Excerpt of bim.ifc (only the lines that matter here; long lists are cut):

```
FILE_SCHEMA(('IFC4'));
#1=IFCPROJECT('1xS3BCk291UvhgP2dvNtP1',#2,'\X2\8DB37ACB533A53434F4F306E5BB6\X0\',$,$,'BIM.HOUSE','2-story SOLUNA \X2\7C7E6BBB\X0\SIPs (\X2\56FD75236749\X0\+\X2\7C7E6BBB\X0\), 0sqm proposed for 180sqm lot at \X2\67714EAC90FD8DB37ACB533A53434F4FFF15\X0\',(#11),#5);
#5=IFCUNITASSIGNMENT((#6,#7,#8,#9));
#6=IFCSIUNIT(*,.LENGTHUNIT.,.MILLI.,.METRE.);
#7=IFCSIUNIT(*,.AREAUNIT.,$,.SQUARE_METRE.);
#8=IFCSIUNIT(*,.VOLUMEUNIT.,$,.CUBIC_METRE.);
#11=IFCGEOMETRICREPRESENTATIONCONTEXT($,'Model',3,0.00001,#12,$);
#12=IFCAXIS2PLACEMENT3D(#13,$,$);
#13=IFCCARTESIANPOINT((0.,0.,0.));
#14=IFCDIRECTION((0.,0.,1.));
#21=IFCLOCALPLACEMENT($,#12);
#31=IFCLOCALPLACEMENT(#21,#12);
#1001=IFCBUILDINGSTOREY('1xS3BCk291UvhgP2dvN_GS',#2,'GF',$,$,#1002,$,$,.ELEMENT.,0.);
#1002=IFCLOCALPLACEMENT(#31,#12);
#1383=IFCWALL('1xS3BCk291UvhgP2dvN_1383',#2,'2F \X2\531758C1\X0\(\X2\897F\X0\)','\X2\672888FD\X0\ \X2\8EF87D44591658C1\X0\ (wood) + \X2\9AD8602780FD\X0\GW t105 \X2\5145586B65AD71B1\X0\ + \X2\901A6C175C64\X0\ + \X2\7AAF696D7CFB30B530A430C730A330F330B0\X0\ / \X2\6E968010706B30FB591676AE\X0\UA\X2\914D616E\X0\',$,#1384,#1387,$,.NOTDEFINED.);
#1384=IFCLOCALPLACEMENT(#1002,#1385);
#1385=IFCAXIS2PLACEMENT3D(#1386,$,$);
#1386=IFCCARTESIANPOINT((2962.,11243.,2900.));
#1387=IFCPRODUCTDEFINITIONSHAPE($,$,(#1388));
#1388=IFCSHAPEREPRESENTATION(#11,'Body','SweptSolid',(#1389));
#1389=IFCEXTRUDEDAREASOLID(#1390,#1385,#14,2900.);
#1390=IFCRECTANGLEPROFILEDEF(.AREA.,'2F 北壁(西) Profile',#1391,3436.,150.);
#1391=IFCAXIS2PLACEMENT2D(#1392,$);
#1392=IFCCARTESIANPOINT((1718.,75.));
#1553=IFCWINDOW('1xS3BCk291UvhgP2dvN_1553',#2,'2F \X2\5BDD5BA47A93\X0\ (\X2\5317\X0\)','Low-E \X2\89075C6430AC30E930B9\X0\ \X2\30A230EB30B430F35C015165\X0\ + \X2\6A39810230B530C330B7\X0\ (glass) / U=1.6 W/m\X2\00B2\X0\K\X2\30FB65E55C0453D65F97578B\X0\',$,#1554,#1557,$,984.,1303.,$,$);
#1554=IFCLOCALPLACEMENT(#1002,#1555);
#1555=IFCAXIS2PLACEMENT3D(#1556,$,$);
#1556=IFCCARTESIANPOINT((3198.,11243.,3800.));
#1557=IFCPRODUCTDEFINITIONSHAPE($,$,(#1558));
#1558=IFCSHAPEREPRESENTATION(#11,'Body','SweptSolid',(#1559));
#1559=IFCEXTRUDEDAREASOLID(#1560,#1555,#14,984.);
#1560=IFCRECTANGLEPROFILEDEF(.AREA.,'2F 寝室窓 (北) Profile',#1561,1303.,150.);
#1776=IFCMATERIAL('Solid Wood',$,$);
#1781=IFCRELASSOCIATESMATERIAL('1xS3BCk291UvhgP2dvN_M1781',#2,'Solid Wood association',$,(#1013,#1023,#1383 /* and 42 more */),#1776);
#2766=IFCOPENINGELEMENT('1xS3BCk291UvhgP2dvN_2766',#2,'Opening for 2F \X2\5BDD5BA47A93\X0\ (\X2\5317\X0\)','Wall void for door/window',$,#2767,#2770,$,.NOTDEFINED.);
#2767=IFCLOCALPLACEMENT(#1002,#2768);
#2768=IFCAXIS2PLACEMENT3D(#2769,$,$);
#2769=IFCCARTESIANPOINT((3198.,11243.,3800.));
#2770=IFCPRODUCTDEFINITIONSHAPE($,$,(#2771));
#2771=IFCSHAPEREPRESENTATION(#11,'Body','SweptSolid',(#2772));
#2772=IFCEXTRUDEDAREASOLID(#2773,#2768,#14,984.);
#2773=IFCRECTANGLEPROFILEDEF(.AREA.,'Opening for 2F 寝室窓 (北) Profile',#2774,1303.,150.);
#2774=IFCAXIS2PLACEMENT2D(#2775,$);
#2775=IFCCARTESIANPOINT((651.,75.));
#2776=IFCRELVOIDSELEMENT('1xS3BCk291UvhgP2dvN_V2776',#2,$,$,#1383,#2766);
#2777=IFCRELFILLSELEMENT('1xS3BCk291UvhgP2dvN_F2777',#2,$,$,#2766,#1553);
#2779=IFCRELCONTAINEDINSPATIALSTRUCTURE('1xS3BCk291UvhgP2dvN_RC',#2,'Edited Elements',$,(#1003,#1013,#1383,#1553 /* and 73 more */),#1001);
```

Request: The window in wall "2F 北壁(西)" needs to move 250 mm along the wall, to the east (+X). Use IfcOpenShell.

```python
import ifcopenshell
import ifcopenshell.api.geometry
import ifcopenshell.util.placement

model = ifcopenshell.open("bim.ifc")

window = model.by_guid("1xS3BCk291UvhgP2dvN_1553")
opening = window.FillsVoids[0].RelatingOpeningElement
wall = opening.VoidsElements[0].RelatingBuildingElement

wall_matrix = ifcopenshell.util.placement.get_local_placement(wall.ObjectPlacement)
shift = wall_matrix[:3, 0] * 250.0
before = ifcopenshell.util.placement.get_local_placement(window.ObjectPlacement)[:3, 3].copy()

# The window is not placed relative to its opening, so move both.
for product in (opening, window):
    matrix = ifcopenshell.util.placement.get_local_placement(product.ObjectPlacement)
    matrix[:3, 3] += shift
    ifcopenshell.api.geometry.edit_object_placement(model, product=product, matrix=matrix, is_si=False)

after = ifcopenshell.util.placement.get_local_placement(window.ObjectPlacement)[:3, 3]
print("window moved by", (after - before).round(3) + 0.0)

model.write("bim_edited.ifc")
```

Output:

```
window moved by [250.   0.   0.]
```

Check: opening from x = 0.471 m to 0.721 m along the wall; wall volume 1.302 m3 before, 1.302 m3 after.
